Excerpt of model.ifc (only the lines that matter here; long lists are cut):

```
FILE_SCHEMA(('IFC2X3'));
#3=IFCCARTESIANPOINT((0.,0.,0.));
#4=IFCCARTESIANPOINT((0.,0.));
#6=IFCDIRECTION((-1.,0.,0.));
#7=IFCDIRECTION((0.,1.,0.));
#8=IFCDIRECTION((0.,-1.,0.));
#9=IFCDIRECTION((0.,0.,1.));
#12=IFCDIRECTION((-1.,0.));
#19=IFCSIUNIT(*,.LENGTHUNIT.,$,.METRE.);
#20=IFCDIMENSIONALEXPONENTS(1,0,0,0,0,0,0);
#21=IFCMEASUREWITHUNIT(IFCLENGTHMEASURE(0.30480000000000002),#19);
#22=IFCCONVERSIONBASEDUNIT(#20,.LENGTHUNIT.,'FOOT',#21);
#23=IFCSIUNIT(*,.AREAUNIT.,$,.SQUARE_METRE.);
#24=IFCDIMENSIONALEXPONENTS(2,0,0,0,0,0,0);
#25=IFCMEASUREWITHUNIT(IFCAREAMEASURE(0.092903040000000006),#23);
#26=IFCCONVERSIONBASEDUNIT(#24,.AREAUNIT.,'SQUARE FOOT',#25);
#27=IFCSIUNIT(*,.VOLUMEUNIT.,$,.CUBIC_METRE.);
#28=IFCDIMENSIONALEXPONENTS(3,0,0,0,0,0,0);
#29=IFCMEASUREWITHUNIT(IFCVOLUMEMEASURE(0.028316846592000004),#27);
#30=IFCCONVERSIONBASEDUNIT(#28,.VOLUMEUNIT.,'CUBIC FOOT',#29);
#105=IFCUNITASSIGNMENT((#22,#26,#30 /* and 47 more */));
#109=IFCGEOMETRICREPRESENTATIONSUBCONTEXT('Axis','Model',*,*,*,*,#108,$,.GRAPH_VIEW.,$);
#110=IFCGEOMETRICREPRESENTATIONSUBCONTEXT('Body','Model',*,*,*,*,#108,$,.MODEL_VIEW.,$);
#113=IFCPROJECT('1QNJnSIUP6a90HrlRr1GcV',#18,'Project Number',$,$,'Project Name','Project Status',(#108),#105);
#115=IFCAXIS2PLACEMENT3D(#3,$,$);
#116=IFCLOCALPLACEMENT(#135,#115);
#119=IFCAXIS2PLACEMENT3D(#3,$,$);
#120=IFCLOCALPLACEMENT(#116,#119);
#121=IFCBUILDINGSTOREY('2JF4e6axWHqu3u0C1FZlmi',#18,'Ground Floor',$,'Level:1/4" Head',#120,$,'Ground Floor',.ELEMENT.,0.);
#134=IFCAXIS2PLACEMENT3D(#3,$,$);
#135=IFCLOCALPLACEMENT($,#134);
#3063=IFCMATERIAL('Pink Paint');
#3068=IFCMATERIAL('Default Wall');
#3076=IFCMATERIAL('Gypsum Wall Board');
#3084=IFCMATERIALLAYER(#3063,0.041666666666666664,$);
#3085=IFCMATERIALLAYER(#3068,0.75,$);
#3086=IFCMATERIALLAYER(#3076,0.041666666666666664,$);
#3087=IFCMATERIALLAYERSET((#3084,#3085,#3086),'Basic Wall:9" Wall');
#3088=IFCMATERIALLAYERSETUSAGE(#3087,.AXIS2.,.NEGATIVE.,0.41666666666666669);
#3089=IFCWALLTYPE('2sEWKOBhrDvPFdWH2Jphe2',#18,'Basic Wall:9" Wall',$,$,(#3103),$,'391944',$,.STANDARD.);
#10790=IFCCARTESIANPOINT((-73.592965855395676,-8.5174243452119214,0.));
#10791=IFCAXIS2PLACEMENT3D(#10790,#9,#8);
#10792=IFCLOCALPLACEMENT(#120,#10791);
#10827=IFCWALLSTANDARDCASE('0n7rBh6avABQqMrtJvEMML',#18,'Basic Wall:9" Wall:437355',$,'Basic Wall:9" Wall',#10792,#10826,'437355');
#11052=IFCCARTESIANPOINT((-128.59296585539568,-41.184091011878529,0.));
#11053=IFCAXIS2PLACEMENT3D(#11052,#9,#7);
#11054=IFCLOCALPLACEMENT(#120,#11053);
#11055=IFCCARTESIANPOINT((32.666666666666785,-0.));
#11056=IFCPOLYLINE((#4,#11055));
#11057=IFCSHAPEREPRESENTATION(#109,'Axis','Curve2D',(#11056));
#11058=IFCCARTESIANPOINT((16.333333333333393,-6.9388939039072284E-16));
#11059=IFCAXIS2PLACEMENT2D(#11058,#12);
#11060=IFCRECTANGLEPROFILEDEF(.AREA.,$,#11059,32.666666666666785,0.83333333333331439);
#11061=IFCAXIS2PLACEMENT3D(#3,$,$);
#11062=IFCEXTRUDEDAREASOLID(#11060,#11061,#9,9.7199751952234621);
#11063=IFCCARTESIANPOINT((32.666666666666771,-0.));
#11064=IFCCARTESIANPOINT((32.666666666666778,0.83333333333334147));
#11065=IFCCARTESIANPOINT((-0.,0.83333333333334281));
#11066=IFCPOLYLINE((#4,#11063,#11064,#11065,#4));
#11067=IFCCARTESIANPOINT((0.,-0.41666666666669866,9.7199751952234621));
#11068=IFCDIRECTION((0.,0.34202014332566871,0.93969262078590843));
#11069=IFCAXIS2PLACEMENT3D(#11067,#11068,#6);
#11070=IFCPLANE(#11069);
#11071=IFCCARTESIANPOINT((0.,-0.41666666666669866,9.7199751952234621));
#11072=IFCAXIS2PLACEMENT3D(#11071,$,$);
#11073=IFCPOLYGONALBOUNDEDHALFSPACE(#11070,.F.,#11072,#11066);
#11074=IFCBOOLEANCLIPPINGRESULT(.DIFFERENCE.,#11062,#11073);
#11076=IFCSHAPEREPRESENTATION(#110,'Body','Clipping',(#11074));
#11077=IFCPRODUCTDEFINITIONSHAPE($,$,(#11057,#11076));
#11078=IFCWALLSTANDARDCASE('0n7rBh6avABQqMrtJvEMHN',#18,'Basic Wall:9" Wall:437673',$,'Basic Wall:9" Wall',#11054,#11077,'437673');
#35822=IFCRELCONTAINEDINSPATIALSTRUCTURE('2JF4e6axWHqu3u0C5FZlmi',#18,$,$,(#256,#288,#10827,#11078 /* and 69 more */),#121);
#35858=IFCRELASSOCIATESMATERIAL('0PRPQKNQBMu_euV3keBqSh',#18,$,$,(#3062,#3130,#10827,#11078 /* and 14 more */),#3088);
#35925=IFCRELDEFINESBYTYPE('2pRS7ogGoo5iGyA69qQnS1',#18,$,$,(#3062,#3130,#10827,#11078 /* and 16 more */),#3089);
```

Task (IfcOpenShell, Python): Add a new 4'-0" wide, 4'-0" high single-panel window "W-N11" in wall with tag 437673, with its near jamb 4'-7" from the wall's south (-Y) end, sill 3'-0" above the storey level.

```python
import numpy as np
import ifcopenshell
import ifcopenshell.api.feature
import ifcopenshell.api.geometry
import ifcopenshell.api.root
import ifcopenshell.api.spatial
import ifcopenshell.api.type
import ifcopenshell.geom
import ifcopenshell.util.element
import ifcopenshell.util.placement
import ifcopenshell.util.representation
import ifcopenshell.util.shape
import ifcopenshell.util.unit

model = ifcopenshell.open("model.ifc")
unit_scale = ifcopenshell.util.unit.calculate_unit_scale(model)
settings = ifcopenshell.geom.settings()


def volume(element):
    """Net volume in cubic metres, openings subtracted."""
    shape = ifcopenshell.geom.create_shape(settings, element)
    return ifcopenshell.util.shape.get_volume(shape.geometry)


wall = model.by_guid("0n7rBh6avABQqMrtJvEMHN")
storey = ifcopenshell.util.element.get_container(wall, ifc_class="IfcBuildingStorey")
context = ifcopenshell.util.representation.get_context(model, "Model", "Body", "MODEL_VIEW")
before = volume(wall)

width, height, from_end, sill = 1.2192, 1.2192, 1.397, 0.9144  # metres

# The wall runs along its own X axis, and the end named is its -X end.
wall_shape = ifcopenshell.geom.create_shape(settings, wall)
x, y, z = ifcopenshell.util.shape.get_vertices(wall_shape.geometry).T
start = x.min() + from_end
face, thickness = float(y.min()), float(y.max() - y.min())
wall_matrix = ifcopenshell.util.placement.get_local_placement(wall.ObjectPlacement)
level = ifcopenshell.util.placement.get_local_placement(storey.ObjectPlacement)[2, 3]


def in_wall(x, y):
    """Placement at x, y metres in the wall's axes, at sill height."""
    matrix = wall_matrix.copy()
    matrix[:, 3] = wall_matrix @ np.array([x / unit_scale, y / unit_scale, 0.0, 1.0])
    matrix[2, 3] = level + sill / unit_scale
    return matrix


# Opening: a box that overshoots both wall faces by 50 mm.
opening = ifcopenshell.api.root.create_entity(model, ifc_class="IfcOpeningElement")
box = ifcopenshell.api.geometry.add_wall_representation(
    model, context=context, length=width, height=height, thickness=thickness + 0.1
)
ifcopenshell.api.geometry.assign_representation(model, product=opening, representation=box)
ifcopenshell.api.geometry.edit_object_placement(model, product=opening, matrix=in_wall(start, face - 0.05), is_si=False)
ifcopenshell.api.feature.add_feature(model, feature=opening, element=wall)

window = ifcopenshell.api.root.create_entity(model, ifc_class="IfcWindow", name="W-N11")
window.OverallWidth, window.OverallHeight = width / unit_scale, height / unit_scale
body = ifcopenshell.api.geometry.add_window_representation(
    model,
    context=context,
    overall_width=window.OverallWidth,
    overall_height=window.OverallHeight,
    partition_type="SINGLE_PANEL",
)
ifcopenshell.api.geometry.assign_representation(model, product=window, representation=body)
ifcopenshell.api.spatial.assign_container(model, products=[window], relating_structure=storey)
fills = ifcopenshell.api.feature.add_filling(model, opening=opening, element=window)
fills.OwnerHistory = window.OwnerHistory  # required in IFC2X3

# IFC2X3 keeps the operation on the window style.
style = ifcopenshell.api.root.create_entity(model, ifc_class="IfcWindowStyle", name="W-N11")
style.OperationType, style.ConstructionType = "SINGLE_PANEL", "NOTDEFINED"
style.ParameterTakesPrecedence = style.Sizeable = False
ifcopenshell.api.type.assign_type(model, related_objects=[window], relating_type=style)

# Centre the window in the wall's thickness.
ifcopenshell.api.geometry.edit_object_placement(model, product=window, matrix=in_wall(start, face), is_si=False)
window_shape = ifcopenshell.geom.create_shape(settings, window)
depth = ifcopenshell.util.shape.get_vertices(window_shape.geometry)[:, 1]
offset = face + thickness / 2 - (depth.min() + depth.max()) / 2
ifcopenshell.api.geometry.edit_object_placement(model, product=window, matrix=in_wall(start, offset), is_si=False)

after = volume(wall)

print(f"wall volume {before:.3f} -> {after:.3f} m3")

model.write("model_updated.ifc")
```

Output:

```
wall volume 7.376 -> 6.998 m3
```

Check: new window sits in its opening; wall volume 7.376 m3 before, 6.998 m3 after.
